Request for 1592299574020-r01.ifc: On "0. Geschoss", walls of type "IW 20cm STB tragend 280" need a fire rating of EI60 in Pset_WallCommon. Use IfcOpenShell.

First a look at what the model holds.

```python
import ifcopenshell
import ifcopenshell.util.element

model = ifcopenshell.open("1592299574020-r01.ifc")
print(model.schema)
storey = next(s for s in model.by_type("IfcBuildingStorey") if s.Name == "0. Geschoss")
walls = [e for e in ifcopenshell.util.element.get_decomposition(storey) if e.is_a("IfcWall")]
seen = {}
for e in walls:
    element_type = ifcopenshell.util.element.get_type(e)
    key = (element_type.Name if element_type != e and element_type else None, ifcopenshell.util.element.get_pset(e, "Pset_WallCommon", "FireRating"))
    seen[key] = seen.get(key, 0) + 1
for (name, value), count in sorted(seen.items(), key=str):
    print(count, "x", name, "|", value)
```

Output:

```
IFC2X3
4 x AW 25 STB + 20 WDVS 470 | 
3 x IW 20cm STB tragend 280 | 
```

```python
import ifcopenshell
import ifcopenshell.api.pset
import ifcopenshell.util.element

model = ifcopenshell.open("1592299574020-r01.ifc")

storey = next(s for s in model.by_type("IfcBuildingStorey") if s.Name == "0. Geschoss")
walls = [e for e in ifcopenshell.util.element.get_decomposition(storey) if e.is_a("IfcWall")]

count = 0
for e in walls:
    element_type = ifcopenshell.util.element.get_type(e)
    if element_type in (None, e) or element_type.Name != "IW 20cm STB tragend 280":
        continue
    # add_pset returns the element's existing set when there is one.
    pset = ifcopenshell.api.pset.add_pset(model, product=e, name="Pset_WallCommon")
    ifcopenshell.api.pset.edit_pset(model, pset=pset, properties={"FireRating": "EI60"})
    count += 1

print(count, "walls updated")

model.write("1592299574020-r01-out.ifc")
```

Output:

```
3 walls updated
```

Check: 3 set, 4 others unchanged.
